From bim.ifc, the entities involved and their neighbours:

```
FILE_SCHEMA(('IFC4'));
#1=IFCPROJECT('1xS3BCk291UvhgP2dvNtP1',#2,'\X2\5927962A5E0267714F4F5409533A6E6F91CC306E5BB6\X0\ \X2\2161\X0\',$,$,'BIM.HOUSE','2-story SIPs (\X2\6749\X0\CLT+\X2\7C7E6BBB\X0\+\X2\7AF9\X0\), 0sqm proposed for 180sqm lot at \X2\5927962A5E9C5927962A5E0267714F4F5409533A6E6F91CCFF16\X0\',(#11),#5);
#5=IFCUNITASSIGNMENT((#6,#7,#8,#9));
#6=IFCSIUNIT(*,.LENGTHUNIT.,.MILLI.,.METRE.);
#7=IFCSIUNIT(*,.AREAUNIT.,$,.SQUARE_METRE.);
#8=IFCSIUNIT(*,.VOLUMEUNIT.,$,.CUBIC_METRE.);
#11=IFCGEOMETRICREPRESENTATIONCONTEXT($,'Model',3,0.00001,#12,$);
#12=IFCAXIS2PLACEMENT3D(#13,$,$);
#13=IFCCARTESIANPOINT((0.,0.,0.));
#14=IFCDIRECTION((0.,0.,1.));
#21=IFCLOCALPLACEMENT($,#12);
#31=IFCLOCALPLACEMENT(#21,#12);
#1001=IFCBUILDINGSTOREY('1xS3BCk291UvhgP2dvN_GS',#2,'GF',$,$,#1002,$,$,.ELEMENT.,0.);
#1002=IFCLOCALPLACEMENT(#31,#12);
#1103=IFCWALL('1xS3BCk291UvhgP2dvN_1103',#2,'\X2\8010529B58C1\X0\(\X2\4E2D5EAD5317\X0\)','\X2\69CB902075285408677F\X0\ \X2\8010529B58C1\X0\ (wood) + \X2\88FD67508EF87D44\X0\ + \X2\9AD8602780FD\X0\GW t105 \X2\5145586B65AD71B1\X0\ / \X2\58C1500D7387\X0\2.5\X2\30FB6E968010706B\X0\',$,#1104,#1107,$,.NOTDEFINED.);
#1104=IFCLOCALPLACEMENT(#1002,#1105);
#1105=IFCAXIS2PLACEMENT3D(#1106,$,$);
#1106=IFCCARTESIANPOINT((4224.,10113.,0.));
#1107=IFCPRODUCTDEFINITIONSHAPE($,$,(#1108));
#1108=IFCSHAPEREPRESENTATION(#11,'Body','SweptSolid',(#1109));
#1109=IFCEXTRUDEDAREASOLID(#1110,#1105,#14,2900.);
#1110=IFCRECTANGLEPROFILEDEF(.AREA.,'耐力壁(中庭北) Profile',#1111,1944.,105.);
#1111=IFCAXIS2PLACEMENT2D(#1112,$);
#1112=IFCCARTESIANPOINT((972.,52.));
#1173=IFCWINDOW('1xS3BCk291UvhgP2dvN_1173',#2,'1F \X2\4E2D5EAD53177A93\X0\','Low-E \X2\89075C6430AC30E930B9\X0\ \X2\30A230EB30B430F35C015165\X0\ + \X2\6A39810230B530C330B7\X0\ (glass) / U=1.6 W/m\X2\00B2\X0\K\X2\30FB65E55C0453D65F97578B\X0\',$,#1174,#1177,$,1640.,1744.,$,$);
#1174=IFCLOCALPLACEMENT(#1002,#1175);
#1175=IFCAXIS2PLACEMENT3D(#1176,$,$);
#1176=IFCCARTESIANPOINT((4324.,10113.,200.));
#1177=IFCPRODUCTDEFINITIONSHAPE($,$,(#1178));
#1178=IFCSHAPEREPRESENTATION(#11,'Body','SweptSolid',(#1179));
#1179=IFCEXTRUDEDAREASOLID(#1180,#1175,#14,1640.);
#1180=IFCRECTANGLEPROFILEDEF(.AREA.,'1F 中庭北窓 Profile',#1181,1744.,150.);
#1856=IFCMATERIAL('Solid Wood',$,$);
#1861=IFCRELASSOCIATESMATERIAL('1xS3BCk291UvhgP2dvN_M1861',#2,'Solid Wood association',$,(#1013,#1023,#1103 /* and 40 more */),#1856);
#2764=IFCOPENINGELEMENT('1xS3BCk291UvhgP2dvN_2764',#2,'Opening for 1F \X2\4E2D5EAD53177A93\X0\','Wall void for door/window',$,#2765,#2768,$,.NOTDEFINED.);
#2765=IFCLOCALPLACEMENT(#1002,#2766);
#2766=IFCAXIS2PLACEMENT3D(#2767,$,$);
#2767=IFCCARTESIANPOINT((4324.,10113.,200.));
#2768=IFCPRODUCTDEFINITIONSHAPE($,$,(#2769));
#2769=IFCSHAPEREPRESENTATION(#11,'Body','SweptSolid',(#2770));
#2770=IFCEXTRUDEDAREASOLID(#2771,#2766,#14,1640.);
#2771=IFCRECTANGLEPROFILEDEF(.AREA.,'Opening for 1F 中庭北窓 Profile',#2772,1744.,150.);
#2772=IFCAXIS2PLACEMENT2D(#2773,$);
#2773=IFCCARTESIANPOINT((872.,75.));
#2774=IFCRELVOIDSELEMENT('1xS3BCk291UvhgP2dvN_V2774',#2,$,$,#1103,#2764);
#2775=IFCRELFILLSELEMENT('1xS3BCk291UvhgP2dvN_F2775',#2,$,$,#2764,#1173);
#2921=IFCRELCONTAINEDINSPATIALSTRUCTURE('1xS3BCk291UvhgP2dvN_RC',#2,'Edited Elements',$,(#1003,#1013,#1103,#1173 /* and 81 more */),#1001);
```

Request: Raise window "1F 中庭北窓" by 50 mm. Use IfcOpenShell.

```python
import numpy as np
import ifcopenshell
import ifcopenshell.api.geometry
import ifcopenshell.util.placement
import ifcopenshell.util.unit

model = ifcopenshell.open("bim.ifc")
unit_scale = ifcopenshell.util.unit.calculate_unit_scale(model)

window = model.by_guid("1xS3BCk291UvhgP2dvN_1173")
opening = window.FillsVoids[0].RelatingOpeningElement
dz = 0.05 / unit_scale

shift = np.array([0.0, 0.0, dz])
# The window is not placed relative to its opening, so move both.
for product in (opening, window):
    matrix = ifcopenshell.util.placement.get_local_placement(product.ObjectPlacement)
    matrix[:3, 3] += shift
    ifcopenshell.api.geometry.edit_object_placement(model, product=product, matrix=matrix, is_si=False)

print(f"moved by {dz * unit_scale:+.3f} m")

model.write("bim_updated.ifc")
```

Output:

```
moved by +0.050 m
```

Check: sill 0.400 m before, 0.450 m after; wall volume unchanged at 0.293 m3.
